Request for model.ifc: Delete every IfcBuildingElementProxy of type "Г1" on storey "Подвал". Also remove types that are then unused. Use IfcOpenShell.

First a look at what the model holds.

```python
import ifcopenshell
import ifcopenshell.util.element

model = ifcopenshell.open("model.ifc")
print(model.schema)
storey = next(s for s in model.by_type("IfcBuildingStorey") if s.Name == "Подвал")
proxies = [e for e in ifcopenshell.util.element.get_decomposition(storey) if e.is_a("IfcBuildingElementProxy")]
seen = {}
for e in proxies:
    element_type = ifcopenshell.util.element.get_type(e)
    name = element_type.Name if element_type not in (None, e) else None
    seen[name] = seen.get(name, 0) + 1
for name, count in sorted(seen.items(), key=str):
    print(count, "x", name)
```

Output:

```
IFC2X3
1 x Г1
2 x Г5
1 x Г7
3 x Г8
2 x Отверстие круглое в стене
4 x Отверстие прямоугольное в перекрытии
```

```python
import ifcopenshell
import ifcopenshell.api.root
import ifcopenshell.util.element

model = ifcopenshell.open("model.ifc")

storey = next(s for s in model.by_type("IfcBuildingStorey") if s.Name == "Подвал")
proxies = [e for e in ifcopenshell.util.element.get_decomposition(storey) if e.is_a("IfcBuildingElementProxy")]
targets = [e for e in proxies if (t := ifcopenshell.util.element.get_type(e)) not in (None, e) and t.Name == "Г1"]
types = {ifcopenshell.util.element.get_type(e) for e in targets} - {None, *targets}

for e in targets:
    ifcopenshell.api.root.remove_product(model, product=e)
print(len(targets), "removed")

unused = [t for t in types if not ifcopenshell.util.element.get_types(t)]
for t in unused:
    ifcopenshell.api.root.remove_product(model, product=t)
print(len(unused), "unused types removed")

model.write("model_rev.ifc")
```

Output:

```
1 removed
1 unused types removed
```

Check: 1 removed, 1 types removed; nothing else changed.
